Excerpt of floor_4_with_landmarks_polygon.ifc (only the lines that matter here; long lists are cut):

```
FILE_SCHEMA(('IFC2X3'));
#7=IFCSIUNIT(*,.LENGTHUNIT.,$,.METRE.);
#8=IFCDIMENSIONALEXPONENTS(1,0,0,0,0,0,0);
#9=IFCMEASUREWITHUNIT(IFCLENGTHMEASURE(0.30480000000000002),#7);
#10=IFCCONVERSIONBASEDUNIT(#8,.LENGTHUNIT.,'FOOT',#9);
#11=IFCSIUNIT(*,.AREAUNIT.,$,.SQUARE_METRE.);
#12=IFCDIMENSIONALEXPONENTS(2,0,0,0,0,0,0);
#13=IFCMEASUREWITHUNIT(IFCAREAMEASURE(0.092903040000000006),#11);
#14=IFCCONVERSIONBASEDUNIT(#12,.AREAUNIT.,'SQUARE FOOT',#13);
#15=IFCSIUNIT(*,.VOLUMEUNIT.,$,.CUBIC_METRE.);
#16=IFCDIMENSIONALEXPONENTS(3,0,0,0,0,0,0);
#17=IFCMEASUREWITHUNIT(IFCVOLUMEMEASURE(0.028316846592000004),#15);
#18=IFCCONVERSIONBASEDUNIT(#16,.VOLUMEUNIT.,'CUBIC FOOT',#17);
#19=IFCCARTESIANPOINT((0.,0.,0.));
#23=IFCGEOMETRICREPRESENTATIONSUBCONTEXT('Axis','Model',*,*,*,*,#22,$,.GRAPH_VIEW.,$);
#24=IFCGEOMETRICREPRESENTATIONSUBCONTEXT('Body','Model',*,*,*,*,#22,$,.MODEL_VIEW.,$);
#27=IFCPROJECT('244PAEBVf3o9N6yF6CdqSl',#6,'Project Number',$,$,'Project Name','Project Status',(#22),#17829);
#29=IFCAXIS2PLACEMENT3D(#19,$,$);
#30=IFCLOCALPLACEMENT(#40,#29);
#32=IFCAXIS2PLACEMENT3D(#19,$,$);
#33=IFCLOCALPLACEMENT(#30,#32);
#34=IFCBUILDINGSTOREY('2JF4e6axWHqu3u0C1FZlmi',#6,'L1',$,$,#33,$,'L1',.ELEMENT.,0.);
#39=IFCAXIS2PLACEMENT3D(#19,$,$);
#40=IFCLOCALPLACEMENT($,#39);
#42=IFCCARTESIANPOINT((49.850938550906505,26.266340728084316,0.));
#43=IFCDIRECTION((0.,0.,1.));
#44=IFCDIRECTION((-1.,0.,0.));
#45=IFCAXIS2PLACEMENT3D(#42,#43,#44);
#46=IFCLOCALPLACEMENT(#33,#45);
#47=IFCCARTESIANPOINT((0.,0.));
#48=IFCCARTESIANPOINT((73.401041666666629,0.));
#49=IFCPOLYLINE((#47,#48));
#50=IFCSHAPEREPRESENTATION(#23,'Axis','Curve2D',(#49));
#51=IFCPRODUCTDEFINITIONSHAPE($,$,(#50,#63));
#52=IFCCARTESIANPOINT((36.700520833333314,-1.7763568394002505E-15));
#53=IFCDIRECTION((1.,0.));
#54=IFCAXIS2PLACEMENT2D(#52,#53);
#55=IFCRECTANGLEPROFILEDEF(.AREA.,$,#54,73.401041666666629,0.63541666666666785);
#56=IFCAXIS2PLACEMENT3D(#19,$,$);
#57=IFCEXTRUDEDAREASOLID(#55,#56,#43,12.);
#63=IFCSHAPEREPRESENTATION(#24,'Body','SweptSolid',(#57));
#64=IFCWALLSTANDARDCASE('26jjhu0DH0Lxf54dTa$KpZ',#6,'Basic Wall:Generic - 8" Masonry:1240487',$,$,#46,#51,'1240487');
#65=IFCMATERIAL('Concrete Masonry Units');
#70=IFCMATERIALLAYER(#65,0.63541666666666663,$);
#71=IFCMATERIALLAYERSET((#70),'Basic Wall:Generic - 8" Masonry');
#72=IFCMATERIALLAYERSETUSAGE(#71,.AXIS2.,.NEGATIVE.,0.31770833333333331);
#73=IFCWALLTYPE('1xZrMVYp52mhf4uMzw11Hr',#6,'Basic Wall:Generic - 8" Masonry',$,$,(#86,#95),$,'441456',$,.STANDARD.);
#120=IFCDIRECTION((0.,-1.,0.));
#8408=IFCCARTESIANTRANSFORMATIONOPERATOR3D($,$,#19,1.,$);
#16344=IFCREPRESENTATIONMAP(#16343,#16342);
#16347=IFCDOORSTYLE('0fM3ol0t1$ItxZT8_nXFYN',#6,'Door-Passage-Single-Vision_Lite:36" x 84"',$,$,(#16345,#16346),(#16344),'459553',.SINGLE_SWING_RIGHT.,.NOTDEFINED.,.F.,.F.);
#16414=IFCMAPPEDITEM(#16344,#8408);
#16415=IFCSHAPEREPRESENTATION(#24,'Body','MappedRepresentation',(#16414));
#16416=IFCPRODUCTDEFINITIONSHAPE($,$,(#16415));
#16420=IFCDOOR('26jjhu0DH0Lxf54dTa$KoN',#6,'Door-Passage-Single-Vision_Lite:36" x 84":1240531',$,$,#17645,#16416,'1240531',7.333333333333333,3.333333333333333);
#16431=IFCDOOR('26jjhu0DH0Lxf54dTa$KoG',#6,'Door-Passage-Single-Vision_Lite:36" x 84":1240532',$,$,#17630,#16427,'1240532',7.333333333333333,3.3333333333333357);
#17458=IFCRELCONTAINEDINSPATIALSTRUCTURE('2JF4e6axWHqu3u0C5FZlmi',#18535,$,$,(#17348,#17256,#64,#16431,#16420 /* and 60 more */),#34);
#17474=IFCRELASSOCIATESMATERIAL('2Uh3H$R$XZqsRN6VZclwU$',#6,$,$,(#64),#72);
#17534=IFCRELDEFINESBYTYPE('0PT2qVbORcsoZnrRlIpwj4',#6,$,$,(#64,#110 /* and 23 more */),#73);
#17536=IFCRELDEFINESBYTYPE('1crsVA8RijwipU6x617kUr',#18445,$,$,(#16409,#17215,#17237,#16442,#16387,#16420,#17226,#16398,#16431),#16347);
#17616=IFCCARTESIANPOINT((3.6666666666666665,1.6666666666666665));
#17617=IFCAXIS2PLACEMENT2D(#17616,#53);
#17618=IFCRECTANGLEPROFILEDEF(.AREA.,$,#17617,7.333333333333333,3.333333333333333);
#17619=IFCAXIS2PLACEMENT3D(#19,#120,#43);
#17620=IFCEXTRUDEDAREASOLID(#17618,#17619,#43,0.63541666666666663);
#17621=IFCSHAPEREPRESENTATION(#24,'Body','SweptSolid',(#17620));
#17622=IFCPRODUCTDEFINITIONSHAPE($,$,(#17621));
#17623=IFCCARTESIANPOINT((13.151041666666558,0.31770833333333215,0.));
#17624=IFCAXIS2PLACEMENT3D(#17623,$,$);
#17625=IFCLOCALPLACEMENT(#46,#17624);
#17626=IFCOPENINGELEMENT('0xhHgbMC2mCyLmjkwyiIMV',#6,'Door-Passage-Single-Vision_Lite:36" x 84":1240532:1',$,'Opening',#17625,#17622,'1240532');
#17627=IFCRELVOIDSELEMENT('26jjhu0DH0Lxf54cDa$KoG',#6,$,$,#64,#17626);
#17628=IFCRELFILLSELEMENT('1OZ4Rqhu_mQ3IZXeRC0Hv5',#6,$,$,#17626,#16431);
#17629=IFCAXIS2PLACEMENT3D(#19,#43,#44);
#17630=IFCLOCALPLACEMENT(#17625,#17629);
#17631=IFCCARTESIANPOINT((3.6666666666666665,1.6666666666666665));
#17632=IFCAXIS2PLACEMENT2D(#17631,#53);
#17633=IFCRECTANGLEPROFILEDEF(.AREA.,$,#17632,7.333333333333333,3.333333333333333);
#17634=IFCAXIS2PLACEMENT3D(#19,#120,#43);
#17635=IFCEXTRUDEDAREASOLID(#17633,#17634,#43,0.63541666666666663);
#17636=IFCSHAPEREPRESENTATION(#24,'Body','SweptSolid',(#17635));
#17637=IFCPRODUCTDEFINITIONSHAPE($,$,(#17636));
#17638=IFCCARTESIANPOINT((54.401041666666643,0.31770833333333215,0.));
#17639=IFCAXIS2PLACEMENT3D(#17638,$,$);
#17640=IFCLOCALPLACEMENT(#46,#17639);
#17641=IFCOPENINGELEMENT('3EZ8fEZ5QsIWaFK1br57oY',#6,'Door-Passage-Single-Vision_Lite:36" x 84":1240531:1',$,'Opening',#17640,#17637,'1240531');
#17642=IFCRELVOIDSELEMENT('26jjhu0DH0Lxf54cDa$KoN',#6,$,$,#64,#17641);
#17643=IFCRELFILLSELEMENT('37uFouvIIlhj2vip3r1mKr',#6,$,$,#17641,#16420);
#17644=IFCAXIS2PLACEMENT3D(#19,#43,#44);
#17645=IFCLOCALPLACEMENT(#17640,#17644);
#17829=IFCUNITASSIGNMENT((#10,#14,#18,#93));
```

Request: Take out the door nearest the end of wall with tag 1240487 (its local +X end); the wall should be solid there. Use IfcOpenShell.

```python
import ifcopenshell
import ifcopenshell.api.feature
import ifcopenshell.api.root
import ifcopenshell.geom
import ifcopenshell.util.shape

model = ifcopenshell.open("floor_4_with_landmarks_polygon.ifc")
settings = ifcopenshell.geom.settings()


def volume(element):
    """Net volume in cubic metres, openings subtracted."""
    shape = ifcopenshell.geom.create_shape(settings, element)
    return ifcopenshell.util.shape.get_volume(shape.geometry)


door = model.by_id(16420)
opening = door.FillsVoids[0].RelatingOpeningElement
wall = opening.VoidsElements[0].RelatingBuildingElement
before = volume(wall)

ifcopenshell.api.root.remove_product(model, product=door)
ifcopenshell.api.feature.remove_feature(model, feature=opening)

after = volume(wall)

print(f"wall volume {before:.3f} -> {after:.3f} m3")

model.write("floor_4_with_landmarks_polygon_edited.ifc")
```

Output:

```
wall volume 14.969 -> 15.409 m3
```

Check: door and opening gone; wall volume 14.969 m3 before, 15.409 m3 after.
